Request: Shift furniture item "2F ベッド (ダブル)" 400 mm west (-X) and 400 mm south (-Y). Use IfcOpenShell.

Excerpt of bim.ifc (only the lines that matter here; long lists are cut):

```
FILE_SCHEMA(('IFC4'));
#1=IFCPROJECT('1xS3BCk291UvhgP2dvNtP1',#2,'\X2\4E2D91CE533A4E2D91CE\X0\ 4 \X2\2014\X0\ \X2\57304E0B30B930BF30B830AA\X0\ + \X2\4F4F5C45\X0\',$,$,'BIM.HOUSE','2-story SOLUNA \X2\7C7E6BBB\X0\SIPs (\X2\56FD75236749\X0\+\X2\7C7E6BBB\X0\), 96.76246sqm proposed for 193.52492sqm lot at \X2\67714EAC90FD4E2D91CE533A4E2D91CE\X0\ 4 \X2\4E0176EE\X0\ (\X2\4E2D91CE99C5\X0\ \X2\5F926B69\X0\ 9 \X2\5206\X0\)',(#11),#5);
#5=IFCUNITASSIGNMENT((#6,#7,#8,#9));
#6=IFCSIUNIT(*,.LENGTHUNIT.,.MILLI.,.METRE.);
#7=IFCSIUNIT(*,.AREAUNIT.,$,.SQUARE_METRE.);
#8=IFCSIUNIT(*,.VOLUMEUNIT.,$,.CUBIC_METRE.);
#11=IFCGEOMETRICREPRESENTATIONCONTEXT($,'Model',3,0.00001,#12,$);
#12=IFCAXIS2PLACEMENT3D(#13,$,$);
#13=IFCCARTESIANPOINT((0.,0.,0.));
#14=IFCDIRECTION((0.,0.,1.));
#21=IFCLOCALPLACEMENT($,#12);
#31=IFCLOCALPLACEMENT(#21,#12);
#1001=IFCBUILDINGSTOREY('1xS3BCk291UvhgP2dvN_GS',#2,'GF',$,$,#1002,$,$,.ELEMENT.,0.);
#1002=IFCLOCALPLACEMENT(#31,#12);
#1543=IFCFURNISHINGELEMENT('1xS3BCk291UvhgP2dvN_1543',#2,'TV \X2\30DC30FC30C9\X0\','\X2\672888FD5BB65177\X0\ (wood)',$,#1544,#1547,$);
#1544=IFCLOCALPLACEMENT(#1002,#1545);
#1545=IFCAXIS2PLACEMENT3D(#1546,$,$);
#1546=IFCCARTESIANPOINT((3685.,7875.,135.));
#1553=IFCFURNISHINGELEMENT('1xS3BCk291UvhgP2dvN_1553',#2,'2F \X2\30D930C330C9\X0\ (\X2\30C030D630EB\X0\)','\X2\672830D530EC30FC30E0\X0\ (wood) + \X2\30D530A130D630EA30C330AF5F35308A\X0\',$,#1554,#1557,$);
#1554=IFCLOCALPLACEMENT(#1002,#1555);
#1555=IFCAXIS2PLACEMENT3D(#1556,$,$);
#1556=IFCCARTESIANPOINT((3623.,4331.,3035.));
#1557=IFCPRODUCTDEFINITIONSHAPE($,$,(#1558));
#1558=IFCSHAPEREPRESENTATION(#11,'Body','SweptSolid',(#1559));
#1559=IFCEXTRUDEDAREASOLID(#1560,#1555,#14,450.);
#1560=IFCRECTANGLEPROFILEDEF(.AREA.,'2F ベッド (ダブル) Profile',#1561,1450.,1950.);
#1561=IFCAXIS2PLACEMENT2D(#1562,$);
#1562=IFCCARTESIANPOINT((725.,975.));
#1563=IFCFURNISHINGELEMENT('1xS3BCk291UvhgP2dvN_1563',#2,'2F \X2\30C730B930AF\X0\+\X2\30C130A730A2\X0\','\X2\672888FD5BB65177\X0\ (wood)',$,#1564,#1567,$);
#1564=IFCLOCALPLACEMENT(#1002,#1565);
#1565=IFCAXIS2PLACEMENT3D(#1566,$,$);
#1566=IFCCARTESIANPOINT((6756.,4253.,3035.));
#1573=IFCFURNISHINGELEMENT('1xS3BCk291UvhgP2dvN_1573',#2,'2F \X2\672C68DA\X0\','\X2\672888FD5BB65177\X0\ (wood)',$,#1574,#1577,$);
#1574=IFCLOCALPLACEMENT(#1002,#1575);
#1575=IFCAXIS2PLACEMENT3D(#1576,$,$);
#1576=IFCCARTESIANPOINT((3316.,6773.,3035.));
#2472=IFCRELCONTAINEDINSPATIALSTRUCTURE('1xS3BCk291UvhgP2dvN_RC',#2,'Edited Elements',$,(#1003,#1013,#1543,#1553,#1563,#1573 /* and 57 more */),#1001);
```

```python
import ifcopenshell
import ifcopenshell.api.geometry
import ifcopenshell.util.placement
import ifcopenshell.util.unit

model = ifcopenshell.open("bim.ifc")
unit_scale = ifcopenshell.util.unit.calculate_unit_scale(model)

item = model.by_guid("1xS3BCk291UvhgP2dvN_1553")
matrix = ifcopenshell.util.placement.get_local_placement(item.ObjectPlacement)
matrix[0, 3] -= 0.4 / unit_scale
matrix[1, 3] -= 0.4 / unit_scale
ifcopenshell.api.geometry.edit_object_placement(model, product=item, matrix=matrix, is_si=False)

print(ifcopenshell.util.placement.get_local_placement(item.ObjectPlacement).round(3) + 0.0)

model.write("bim-out.ifc")
```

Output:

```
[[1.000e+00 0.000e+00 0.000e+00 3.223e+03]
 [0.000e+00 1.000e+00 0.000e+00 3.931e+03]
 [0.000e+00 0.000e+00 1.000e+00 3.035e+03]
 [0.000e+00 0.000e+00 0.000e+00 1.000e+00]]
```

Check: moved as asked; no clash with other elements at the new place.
